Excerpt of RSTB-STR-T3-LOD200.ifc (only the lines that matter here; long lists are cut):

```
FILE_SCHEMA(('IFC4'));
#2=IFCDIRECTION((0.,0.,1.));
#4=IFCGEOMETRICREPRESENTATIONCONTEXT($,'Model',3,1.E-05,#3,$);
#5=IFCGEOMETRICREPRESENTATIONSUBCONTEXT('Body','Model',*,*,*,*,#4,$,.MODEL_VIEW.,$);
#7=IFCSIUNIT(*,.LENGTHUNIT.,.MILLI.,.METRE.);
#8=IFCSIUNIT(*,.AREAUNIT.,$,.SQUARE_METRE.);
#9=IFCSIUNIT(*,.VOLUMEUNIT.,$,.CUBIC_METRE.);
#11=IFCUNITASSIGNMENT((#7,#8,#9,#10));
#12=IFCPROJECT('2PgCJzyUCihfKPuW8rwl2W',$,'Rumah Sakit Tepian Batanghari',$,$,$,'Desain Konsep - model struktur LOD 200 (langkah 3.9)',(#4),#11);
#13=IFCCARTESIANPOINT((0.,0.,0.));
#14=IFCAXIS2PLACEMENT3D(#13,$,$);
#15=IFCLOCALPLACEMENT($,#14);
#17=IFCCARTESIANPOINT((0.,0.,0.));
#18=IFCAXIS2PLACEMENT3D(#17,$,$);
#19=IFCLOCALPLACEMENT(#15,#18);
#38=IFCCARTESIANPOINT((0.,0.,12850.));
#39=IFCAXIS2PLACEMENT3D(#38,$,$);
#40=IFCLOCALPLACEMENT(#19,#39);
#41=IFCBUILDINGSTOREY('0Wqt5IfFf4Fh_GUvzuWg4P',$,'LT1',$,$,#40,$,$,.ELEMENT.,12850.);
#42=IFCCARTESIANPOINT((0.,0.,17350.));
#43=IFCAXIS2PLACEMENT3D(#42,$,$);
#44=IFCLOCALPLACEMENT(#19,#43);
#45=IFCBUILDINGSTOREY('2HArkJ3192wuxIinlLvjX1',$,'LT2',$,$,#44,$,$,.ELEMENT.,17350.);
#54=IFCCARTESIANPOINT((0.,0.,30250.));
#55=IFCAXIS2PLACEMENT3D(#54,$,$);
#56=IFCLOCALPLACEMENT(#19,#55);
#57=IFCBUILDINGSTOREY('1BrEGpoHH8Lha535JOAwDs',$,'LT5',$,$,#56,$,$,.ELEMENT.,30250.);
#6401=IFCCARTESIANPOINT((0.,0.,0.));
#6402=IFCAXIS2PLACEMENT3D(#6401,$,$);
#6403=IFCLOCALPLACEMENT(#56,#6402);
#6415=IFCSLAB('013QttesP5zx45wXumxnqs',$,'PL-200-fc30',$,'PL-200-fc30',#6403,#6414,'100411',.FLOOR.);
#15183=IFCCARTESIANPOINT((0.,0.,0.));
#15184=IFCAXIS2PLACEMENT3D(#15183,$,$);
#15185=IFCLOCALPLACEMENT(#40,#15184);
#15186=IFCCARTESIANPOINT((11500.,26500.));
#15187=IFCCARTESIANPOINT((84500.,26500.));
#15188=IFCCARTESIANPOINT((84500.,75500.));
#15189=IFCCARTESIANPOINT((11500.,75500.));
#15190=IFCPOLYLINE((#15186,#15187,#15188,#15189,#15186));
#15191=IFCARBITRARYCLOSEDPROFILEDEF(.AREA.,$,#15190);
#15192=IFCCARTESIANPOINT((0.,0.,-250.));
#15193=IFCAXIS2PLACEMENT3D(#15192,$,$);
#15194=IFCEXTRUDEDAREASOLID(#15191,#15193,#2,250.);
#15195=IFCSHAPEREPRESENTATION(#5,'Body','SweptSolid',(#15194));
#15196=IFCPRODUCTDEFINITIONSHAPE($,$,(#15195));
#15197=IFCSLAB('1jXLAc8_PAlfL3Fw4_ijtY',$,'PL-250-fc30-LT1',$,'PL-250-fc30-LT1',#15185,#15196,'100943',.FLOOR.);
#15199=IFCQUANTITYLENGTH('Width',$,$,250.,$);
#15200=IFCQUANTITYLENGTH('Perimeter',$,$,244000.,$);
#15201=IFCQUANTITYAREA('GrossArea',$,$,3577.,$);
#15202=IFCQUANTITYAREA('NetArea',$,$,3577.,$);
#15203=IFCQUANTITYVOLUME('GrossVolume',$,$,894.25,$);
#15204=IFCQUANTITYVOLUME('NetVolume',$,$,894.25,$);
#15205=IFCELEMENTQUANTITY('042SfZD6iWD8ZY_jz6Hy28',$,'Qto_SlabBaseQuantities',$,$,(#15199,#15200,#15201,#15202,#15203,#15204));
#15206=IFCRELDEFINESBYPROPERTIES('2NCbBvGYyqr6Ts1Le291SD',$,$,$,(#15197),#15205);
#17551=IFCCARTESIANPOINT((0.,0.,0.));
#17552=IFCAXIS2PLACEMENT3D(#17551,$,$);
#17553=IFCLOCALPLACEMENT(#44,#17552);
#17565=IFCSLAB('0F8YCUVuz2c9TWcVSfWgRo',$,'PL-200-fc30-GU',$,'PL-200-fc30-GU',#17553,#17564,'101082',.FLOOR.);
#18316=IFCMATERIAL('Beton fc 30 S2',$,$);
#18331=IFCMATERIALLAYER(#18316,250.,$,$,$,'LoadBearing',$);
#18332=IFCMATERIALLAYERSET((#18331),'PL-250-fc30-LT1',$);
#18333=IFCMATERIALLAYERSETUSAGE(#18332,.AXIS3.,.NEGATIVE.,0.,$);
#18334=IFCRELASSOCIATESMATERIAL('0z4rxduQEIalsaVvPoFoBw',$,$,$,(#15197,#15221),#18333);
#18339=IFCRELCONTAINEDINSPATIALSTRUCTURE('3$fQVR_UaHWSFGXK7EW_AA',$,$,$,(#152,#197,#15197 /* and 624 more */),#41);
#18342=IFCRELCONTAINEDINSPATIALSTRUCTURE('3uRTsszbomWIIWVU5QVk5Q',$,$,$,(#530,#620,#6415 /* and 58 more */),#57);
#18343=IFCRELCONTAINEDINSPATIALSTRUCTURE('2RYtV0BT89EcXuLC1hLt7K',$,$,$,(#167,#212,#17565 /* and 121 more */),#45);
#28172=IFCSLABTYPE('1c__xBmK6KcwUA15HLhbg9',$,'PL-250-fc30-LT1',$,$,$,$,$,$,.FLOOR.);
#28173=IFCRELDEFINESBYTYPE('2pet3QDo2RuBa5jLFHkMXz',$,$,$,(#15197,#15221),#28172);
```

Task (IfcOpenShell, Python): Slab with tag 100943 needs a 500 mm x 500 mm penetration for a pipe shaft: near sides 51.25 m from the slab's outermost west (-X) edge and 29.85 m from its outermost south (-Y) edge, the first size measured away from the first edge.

```python
import numpy as np
import ifcopenshell
import ifcopenshell.api.feature
import ifcopenshell.api.geometry
import ifcopenshell.api.pset
import ifcopenshell.api.root
import ifcopenshell.geom
import ifcopenshell.util.element
import ifcopenshell.util.placement
import ifcopenshell.util.representation
import ifcopenshell.util.shape
import ifcopenshell.util.unit

model = ifcopenshell.open("RSTB-STR-T3-LOD200.ifc")
unit_scale = ifcopenshell.util.unit.calculate_unit_scale(model)
area_scale = ifcopenshell.util.unit.calculate_unit_scale(model, "AREAUNIT")
volume_scale = ifcopenshell.util.unit.calculate_unit_scale(model, "VOLUMEUNIT")
settings = ifcopenshell.geom.settings()


def volume(element):
    """Net volume in cubic metres, openings subtracted."""
    shape = ifcopenshell.geom.create_shape(settings, element)
    return ifcopenshell.util.shape.get_volume(shape.geometry)


slab = model.by_id(15197)
before = volume(slab)

# Extent in the slab's own axes, in metres. The edges named are its -X and -Y sides.
slab_shape = ifcopenshell.geom.create_shape(settings, slab)
vertices = ifcopenshell.util.shape.get_vertices(slab_shape.geometry)
x_min, y_min, bottom = vertices.min(axis=0)
top = vertices[:, 2].max()

opening = ifcopenshell.api.root.create_entity(model, ifc_class="IfcOpeningElement", name="Pipe shaft opening", predefined_type="OPENING")
context = ifcopenshell.util.representation.get_context(model, "Model", "Body", "MODEL_VIEW")
width, depth = 0.5, 0.5
outline = [(0.0, 0.0), (width, 0.0), (width, depth), (0.0, depth), (0.0, 0.0)]
# Overshoot both faces by 50 mm so the cut is clean.
shape = ifcopenshell.api.geometry.add_slab_representation(
    model, context=context, depth=top - bottom + 0.1, polyline=outline
)
ifcopenshell.api.geometry.assign_representation(model, product=opening, representation=shape)

matrix = ifcopenshell.util.placement.get_local_placement(slab.ObjectPlacement)
matrix[:, 3] = matrix @ np.append(np.array([x_min + 51.25, y_min + 29.85, bottom - 0.05]) / unit_scale, 1.0)
ifcopenshell.api.geometry.edit_object_placement(model, product=opening, matrix=matrix, is_si=False)
ifcopenshell.api.feature.add_feature(model, feature=opening, element=slab)

after = volume(slab)

# Update the slab's stored quantities.
qto = model.by_id(ifcopenshell.util.element.get_pset(slab, "Qto_SlabBaseQuantities", should_inherit=False)["id"])
ifcopenshell.api.pset.edit_qto(model, qto=qto, properties={
    "NetArea": after / (top - bottom) / area_scale,
    "NetVolume": after / volume_scale,
})

print(f"slab volume {before:.3f} -> {after:.3f} m3")

model.write("RSTB-STR-T3-LOD200_updated.ifc")
```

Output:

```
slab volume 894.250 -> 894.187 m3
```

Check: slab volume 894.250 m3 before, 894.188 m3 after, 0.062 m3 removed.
